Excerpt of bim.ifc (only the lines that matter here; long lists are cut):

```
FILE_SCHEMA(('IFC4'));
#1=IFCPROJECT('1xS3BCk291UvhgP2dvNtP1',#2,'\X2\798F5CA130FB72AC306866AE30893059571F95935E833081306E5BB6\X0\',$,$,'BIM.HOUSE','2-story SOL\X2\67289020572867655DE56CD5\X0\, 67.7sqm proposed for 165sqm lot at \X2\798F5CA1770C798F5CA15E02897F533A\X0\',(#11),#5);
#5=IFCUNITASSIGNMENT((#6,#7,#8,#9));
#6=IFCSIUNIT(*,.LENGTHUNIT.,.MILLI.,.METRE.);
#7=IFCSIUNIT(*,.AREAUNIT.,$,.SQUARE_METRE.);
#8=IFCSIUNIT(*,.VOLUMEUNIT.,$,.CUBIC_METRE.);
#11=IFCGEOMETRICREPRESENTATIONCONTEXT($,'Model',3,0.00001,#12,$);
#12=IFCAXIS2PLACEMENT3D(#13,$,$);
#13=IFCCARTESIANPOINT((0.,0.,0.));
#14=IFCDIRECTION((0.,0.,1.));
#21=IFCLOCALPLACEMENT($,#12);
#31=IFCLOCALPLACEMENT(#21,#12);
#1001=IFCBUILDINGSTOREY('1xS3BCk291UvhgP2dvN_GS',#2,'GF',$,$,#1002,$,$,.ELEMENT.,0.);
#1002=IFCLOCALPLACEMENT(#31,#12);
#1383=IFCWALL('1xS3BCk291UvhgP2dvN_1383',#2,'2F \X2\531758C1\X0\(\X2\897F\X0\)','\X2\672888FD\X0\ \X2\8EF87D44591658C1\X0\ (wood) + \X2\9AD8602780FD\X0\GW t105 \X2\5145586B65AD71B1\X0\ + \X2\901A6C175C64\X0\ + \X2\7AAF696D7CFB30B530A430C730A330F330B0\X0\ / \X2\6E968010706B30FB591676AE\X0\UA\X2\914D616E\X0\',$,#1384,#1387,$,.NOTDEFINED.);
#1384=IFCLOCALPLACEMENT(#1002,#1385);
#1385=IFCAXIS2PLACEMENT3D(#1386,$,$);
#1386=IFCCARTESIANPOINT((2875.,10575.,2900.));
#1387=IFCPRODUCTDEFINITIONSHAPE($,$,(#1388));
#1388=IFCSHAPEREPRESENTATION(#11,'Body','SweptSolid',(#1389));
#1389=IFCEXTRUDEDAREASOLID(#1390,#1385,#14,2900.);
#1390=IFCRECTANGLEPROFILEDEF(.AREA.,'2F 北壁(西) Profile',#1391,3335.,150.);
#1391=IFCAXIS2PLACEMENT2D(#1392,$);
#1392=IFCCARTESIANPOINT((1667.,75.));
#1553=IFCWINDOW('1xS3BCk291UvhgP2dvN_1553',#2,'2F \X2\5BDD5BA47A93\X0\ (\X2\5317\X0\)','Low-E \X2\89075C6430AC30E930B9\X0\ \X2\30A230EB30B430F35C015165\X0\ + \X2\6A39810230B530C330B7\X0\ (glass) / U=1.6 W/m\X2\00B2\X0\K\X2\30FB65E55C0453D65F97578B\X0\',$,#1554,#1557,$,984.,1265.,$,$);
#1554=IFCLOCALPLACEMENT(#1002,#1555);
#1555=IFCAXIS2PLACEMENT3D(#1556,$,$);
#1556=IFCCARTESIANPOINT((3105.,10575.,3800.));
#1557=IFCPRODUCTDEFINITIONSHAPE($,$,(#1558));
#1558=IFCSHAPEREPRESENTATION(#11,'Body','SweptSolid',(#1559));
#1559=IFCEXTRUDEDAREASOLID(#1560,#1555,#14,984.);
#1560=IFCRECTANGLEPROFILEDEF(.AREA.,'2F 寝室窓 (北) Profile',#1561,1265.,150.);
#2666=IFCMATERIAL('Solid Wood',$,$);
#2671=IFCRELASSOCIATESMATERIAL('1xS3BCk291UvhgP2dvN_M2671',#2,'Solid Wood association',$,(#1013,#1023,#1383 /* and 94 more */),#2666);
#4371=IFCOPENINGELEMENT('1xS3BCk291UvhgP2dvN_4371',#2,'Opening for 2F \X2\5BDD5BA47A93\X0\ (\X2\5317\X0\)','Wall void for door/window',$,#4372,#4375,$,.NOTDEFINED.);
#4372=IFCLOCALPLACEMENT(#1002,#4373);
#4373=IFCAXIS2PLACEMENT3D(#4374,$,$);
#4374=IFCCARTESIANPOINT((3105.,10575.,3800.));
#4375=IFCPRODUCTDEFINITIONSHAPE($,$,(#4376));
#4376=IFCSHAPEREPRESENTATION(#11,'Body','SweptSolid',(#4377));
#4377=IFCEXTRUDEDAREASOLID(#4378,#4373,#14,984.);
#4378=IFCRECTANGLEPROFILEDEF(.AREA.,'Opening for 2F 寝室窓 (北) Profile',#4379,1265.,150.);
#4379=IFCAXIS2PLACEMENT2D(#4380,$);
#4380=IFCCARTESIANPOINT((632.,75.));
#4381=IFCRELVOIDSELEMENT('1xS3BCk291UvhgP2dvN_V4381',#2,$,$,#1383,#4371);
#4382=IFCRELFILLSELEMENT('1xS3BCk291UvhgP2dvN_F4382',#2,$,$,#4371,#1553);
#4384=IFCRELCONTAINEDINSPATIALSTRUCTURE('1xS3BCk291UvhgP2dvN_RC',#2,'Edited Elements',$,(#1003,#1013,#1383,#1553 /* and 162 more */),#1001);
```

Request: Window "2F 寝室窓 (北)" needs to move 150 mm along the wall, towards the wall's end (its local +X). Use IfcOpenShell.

```python
import ifcopenshell
import ifcopenshell.api.geometry
import ifcopenshell.util.placement
import ifcopenshell.util.unit

model = ifcopenshell.open("bim.ifc")
unit_scale = ifcopenshell.util.unit.calculate_unit_scale(model)

window = model.by_guid("1xS3BCk291UvhgP2dvN_1553")
opening = window.FillsVoids[0].RelatingOpeningElement
wall = opening.VoidsElements[0].RelatingBuildingElement

wall_matrix = ifcopenshell.util.placement.get_local_placement(wall.ObjectPlacement)
shift = wall_matrix[:3, 0] * 0.15 / unit_scale
before = ifcopenshell.util.placement.get_local_placement(window.ObjectPlacement)[:3, 3].copy()

# The window is not placed relative to its opening, so move both.
for product in (opening, window):
    matrix = ifcopenshell.util.placement.get_local_placement(product.ObjectPlacement)
    matrix[:3, 3] += shift
    ifcopenshell.api.geometry.edit_object_placement(model, product=product, matrix=matrix, is_si=False)

after = ifcopenshell.util.placement.get_local_placement(window.ObjectPlacement)[:3, 3]
print("window moved by", (after - before).round(3) + 0.0)

model.write("bim_v2.ifc")
```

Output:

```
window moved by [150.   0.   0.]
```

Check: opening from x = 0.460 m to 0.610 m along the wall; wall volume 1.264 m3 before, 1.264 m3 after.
